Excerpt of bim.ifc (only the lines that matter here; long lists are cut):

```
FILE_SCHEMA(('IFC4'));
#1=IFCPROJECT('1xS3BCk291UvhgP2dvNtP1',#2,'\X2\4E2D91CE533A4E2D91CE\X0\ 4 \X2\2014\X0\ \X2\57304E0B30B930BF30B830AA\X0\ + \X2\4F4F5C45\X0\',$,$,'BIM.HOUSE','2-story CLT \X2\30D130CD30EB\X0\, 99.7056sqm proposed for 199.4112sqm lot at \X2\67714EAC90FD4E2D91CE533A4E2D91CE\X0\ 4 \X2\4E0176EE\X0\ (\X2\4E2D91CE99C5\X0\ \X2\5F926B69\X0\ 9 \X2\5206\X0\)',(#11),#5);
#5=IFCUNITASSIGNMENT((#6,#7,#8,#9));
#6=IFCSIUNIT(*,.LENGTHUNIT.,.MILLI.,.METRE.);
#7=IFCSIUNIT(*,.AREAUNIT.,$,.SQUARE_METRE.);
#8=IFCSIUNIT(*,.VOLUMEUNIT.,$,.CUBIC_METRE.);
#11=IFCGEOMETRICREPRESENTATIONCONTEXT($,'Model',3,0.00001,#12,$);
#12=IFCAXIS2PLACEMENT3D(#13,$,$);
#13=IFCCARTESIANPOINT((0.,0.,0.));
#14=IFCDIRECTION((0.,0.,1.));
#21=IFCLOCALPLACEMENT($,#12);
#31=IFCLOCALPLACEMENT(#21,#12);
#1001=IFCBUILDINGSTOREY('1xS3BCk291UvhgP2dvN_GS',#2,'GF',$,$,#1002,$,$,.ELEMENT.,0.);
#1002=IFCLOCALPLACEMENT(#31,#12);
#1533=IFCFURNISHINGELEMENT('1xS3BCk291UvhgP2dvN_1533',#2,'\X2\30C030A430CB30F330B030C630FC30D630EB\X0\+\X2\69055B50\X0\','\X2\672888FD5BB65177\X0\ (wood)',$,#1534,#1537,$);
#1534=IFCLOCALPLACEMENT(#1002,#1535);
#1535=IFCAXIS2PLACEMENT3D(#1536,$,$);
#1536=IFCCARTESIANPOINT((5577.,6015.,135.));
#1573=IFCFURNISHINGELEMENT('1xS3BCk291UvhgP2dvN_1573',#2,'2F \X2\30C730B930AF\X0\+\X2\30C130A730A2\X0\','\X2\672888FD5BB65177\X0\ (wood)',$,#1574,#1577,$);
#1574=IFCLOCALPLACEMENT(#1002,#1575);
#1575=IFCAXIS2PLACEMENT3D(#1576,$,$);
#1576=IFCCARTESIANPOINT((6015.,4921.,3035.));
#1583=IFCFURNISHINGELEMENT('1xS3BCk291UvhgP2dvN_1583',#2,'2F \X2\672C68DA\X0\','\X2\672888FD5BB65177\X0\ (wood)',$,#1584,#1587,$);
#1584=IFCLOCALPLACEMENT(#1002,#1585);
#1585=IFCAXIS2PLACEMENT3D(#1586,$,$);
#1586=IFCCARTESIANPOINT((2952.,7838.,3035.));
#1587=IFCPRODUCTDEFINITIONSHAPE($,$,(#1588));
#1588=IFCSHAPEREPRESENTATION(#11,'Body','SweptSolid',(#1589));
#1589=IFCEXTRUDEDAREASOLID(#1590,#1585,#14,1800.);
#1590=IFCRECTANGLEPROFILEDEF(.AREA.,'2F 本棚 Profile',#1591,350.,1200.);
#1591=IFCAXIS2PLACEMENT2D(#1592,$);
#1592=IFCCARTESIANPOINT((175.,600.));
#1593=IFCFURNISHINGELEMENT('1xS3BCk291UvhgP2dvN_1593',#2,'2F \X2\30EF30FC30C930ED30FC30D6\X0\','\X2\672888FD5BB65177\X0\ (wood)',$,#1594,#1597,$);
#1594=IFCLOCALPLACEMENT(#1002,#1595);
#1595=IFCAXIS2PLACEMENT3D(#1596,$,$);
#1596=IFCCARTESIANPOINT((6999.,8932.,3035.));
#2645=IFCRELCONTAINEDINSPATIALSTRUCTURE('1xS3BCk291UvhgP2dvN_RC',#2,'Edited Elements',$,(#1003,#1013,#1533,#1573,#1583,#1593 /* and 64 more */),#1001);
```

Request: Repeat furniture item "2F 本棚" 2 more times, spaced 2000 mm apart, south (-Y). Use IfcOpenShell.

```python
import numpy as np
import ifcopenshell
import ifcopenshell.api.geometry
import ifcopenshell.api.root
import ifcopenshell.util.element
import ifcopenshell.util.placement
import ifcopenshell.util.unit

model = ifcopenshell.open("bim.ifc")
unit_scale = ifcopenshell.util.unit.calculate_unit_scale(model)


def reuse_history(source, copy):
    """copy_class also copies each property set's owner history, people and application; keep the originals."""
    for rel in copy.IsDefinedBy:
        if rel.is_a("IfcRelDefinesByProperties") and (history := rel.RelatingPropertyDefinition.OwnerHistory):
            rel.RelatingPropertyDefinition.OwnerHistory = source.OwnerHistory
            ifcopenshell.util.element.remove_deep2(model, history)


source = model.by_guid("1xS3BCk291UvhgP2dvN_1583")
base = ifcopenshell.util.placement.get_local_placement(source.ObjectPlacement)
step = np.array([0.0, -1.0, 0.0]) * 2 / unit_scale

for i in range(1, 3):
    copy = ifcopenshell.api.root.copy_class(model, product=source)
    copy.Representation = ifcopenshell.util.element.copy_deep(
        model, source.Representation, exclude=["IfcGeometricRepresentationContext", "IfcRepresentationMap"]
    )
    reuse_history(source, copy)
    matrix = base.copy()
    matrix[:3, 3] += i * step
    print("added at", matrix[:3, 3].round(3) + 0.0)
    ifcopenshell.api.geometry.edit_object_placement(model, product=copy, matrix=matrix, is_si=False)

model.write("bim_v2.ifc")
```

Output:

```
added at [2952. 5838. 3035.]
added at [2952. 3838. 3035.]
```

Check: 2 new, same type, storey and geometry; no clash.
